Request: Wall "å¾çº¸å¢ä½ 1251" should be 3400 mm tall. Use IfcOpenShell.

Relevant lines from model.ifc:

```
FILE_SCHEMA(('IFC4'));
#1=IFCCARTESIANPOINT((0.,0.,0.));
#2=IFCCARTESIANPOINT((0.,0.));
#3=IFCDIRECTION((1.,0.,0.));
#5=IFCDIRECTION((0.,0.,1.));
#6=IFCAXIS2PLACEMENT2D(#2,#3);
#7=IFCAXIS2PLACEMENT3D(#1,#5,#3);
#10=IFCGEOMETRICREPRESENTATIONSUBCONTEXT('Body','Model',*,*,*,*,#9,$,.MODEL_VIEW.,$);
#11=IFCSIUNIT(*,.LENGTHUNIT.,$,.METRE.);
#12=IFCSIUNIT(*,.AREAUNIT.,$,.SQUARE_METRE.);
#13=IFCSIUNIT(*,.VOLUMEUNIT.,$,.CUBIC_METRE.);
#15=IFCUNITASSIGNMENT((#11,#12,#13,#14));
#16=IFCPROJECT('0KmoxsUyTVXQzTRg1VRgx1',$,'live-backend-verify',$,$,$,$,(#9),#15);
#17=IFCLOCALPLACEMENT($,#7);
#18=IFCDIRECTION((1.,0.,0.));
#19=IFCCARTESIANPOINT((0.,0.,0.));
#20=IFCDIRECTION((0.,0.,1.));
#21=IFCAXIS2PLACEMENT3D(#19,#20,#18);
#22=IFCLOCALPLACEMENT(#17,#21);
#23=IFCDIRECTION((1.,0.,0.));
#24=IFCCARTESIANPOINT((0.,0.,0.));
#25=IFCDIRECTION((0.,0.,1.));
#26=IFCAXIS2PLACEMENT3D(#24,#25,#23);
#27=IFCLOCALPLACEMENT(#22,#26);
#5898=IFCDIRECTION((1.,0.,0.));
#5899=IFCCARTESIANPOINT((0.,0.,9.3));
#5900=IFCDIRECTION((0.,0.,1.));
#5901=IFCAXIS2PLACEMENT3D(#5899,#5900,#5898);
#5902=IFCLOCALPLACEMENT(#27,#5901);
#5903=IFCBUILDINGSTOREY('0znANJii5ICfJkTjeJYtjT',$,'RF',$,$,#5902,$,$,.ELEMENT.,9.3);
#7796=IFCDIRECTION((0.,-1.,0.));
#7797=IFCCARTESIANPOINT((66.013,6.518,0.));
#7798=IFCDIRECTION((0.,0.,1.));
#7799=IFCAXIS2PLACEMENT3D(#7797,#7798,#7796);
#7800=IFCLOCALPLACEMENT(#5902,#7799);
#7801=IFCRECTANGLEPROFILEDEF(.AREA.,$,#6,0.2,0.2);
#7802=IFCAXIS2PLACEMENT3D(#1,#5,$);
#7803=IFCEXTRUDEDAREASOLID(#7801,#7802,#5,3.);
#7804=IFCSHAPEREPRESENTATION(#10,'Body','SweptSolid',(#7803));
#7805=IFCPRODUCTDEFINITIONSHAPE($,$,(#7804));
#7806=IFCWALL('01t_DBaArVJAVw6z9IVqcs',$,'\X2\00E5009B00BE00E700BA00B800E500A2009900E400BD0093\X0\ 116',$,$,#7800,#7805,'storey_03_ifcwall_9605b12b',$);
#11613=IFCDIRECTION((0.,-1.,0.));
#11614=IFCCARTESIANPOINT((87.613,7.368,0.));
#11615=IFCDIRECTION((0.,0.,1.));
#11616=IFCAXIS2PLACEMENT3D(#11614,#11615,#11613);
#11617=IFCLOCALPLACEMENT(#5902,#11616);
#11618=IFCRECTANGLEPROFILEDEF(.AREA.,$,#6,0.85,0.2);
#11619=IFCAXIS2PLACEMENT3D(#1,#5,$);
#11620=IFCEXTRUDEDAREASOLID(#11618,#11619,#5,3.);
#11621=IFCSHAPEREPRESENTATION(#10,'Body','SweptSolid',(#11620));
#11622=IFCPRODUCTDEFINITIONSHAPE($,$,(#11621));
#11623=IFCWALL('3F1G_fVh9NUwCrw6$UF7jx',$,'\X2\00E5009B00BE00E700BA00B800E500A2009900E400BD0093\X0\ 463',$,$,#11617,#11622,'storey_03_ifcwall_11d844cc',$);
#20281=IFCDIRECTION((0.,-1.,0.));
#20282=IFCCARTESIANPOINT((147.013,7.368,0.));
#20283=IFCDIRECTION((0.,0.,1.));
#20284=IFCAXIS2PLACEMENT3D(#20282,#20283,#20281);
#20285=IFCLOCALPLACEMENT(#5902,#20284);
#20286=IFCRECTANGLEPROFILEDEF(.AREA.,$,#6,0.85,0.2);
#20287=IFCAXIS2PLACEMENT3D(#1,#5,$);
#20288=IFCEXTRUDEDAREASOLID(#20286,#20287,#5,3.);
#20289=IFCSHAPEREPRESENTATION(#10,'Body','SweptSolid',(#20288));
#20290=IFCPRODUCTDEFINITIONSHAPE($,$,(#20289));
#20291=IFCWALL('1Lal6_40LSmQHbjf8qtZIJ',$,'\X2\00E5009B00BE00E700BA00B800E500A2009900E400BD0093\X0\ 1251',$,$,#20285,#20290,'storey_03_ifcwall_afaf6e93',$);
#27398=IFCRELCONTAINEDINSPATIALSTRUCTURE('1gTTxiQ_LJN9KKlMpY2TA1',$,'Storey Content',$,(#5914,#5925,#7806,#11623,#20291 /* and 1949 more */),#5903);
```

```python
import ifcopenshell
import ifcopenshell.geom
import ifcopenshell.util.representation
import ifcopenshell.util.shape
import ifcopenshell.util.unit

model = ifcopenshell.open("model.ifc")
unit_scale = ifcopenshell.util.unit.calculate_unit_scale(model)
settings = ifcopenshell.geom.settings()


def volume(element):
    """Net volume in cubic metres, openings subtracted."""
    shape = ifcopenshell.geom.create_shape(settings, element)
    return ifcopenshell.util.shape.get_volume(shape.geometry)


wall = model.by_id(20291)
before = volume(wall)

body = ifcopenshell.util.representation.get_representation(wall, "Model", "Body")
solid = body.Items[0]
old_height = solid.Depth
solid.Depth = 3.4 / unit_scale
after = volume(wall)

print(f"height {old_height:g} -> {solid.Depth:g}, volume {before:.3f} -> {after:.3f} m3")

model.write("model_edited.ifc")
```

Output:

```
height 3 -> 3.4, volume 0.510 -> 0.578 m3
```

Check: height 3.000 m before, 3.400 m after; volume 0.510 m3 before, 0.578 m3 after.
